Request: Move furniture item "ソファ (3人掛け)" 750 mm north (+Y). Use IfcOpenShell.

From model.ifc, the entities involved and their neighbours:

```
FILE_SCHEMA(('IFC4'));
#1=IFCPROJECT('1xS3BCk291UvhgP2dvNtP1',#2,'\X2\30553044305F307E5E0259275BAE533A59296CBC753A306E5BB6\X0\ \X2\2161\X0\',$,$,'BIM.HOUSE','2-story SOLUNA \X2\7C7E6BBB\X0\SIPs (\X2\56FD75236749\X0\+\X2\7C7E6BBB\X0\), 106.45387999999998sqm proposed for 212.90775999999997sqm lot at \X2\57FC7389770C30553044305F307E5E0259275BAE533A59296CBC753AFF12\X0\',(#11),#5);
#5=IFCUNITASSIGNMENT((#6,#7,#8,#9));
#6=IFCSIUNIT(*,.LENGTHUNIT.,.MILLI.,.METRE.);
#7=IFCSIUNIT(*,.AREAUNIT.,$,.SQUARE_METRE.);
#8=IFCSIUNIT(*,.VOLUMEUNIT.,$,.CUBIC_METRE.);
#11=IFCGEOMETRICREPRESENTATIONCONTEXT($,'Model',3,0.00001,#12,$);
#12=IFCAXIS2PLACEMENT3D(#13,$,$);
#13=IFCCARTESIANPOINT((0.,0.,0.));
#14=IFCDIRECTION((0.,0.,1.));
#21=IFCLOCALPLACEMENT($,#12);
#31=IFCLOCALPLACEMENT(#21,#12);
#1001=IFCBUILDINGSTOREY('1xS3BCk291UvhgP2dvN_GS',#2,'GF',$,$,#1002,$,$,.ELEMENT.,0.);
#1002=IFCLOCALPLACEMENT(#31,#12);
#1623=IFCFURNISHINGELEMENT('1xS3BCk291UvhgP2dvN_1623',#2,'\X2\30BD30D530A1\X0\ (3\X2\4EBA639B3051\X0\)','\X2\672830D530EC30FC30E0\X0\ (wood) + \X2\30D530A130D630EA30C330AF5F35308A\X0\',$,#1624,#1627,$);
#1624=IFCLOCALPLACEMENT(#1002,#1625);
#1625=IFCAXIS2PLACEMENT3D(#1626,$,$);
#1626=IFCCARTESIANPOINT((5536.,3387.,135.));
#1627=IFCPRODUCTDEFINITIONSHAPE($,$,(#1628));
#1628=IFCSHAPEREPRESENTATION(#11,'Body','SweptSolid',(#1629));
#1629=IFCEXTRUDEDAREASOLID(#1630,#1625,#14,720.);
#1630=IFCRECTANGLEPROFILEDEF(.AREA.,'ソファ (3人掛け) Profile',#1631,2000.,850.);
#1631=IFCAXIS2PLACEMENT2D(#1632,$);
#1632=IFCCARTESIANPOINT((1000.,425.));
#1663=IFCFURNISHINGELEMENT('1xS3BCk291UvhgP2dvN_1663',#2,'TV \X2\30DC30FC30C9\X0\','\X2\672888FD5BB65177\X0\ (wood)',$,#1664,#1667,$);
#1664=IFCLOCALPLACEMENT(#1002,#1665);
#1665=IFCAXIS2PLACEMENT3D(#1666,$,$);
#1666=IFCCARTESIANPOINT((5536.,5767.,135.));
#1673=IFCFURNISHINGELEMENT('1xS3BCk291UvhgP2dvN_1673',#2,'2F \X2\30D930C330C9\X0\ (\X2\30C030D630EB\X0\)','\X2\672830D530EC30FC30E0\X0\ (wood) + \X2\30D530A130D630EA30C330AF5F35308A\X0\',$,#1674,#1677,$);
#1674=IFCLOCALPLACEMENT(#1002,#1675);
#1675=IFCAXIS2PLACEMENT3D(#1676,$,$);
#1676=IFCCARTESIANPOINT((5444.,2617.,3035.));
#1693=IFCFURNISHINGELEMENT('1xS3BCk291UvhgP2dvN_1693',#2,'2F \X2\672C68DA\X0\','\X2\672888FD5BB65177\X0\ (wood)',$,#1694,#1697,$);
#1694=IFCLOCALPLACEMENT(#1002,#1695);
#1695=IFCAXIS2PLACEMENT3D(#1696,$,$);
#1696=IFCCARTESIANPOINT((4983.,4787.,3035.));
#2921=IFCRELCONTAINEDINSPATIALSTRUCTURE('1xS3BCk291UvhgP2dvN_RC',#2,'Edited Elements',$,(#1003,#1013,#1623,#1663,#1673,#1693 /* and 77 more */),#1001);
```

```python
import ifcopenshell
import ifcopenshell.api.geometry
import ifcopenshell.util.placement
import ifcopenshell.util.unit

model = ifcopenshell.open("model.ifc")
unit_scale = ifcopenshell.util.unit.calculate_unit_scale(model)

item = model.by_guid("1xS3BCk291UvhgP2dvN_1623")
matrix = ifcopenshell.util.placement.get_local_placement(item.ObjectPlacement)
matrix[1, 3] += 0.75 / unit_scale
ifcopenshell.api.geometry.edit_object_placement(model, product=item, matrix=matrix, is_si=False)

print(ifcopenshell.util.placement.get_local_placement(item.ObjectPlacement).round(3) + 0.0)

model.write("model-out.ifc")
```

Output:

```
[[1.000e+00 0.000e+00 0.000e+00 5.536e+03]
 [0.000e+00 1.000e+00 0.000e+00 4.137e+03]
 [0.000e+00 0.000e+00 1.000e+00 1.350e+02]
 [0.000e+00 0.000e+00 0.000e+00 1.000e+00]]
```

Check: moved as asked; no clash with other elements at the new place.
